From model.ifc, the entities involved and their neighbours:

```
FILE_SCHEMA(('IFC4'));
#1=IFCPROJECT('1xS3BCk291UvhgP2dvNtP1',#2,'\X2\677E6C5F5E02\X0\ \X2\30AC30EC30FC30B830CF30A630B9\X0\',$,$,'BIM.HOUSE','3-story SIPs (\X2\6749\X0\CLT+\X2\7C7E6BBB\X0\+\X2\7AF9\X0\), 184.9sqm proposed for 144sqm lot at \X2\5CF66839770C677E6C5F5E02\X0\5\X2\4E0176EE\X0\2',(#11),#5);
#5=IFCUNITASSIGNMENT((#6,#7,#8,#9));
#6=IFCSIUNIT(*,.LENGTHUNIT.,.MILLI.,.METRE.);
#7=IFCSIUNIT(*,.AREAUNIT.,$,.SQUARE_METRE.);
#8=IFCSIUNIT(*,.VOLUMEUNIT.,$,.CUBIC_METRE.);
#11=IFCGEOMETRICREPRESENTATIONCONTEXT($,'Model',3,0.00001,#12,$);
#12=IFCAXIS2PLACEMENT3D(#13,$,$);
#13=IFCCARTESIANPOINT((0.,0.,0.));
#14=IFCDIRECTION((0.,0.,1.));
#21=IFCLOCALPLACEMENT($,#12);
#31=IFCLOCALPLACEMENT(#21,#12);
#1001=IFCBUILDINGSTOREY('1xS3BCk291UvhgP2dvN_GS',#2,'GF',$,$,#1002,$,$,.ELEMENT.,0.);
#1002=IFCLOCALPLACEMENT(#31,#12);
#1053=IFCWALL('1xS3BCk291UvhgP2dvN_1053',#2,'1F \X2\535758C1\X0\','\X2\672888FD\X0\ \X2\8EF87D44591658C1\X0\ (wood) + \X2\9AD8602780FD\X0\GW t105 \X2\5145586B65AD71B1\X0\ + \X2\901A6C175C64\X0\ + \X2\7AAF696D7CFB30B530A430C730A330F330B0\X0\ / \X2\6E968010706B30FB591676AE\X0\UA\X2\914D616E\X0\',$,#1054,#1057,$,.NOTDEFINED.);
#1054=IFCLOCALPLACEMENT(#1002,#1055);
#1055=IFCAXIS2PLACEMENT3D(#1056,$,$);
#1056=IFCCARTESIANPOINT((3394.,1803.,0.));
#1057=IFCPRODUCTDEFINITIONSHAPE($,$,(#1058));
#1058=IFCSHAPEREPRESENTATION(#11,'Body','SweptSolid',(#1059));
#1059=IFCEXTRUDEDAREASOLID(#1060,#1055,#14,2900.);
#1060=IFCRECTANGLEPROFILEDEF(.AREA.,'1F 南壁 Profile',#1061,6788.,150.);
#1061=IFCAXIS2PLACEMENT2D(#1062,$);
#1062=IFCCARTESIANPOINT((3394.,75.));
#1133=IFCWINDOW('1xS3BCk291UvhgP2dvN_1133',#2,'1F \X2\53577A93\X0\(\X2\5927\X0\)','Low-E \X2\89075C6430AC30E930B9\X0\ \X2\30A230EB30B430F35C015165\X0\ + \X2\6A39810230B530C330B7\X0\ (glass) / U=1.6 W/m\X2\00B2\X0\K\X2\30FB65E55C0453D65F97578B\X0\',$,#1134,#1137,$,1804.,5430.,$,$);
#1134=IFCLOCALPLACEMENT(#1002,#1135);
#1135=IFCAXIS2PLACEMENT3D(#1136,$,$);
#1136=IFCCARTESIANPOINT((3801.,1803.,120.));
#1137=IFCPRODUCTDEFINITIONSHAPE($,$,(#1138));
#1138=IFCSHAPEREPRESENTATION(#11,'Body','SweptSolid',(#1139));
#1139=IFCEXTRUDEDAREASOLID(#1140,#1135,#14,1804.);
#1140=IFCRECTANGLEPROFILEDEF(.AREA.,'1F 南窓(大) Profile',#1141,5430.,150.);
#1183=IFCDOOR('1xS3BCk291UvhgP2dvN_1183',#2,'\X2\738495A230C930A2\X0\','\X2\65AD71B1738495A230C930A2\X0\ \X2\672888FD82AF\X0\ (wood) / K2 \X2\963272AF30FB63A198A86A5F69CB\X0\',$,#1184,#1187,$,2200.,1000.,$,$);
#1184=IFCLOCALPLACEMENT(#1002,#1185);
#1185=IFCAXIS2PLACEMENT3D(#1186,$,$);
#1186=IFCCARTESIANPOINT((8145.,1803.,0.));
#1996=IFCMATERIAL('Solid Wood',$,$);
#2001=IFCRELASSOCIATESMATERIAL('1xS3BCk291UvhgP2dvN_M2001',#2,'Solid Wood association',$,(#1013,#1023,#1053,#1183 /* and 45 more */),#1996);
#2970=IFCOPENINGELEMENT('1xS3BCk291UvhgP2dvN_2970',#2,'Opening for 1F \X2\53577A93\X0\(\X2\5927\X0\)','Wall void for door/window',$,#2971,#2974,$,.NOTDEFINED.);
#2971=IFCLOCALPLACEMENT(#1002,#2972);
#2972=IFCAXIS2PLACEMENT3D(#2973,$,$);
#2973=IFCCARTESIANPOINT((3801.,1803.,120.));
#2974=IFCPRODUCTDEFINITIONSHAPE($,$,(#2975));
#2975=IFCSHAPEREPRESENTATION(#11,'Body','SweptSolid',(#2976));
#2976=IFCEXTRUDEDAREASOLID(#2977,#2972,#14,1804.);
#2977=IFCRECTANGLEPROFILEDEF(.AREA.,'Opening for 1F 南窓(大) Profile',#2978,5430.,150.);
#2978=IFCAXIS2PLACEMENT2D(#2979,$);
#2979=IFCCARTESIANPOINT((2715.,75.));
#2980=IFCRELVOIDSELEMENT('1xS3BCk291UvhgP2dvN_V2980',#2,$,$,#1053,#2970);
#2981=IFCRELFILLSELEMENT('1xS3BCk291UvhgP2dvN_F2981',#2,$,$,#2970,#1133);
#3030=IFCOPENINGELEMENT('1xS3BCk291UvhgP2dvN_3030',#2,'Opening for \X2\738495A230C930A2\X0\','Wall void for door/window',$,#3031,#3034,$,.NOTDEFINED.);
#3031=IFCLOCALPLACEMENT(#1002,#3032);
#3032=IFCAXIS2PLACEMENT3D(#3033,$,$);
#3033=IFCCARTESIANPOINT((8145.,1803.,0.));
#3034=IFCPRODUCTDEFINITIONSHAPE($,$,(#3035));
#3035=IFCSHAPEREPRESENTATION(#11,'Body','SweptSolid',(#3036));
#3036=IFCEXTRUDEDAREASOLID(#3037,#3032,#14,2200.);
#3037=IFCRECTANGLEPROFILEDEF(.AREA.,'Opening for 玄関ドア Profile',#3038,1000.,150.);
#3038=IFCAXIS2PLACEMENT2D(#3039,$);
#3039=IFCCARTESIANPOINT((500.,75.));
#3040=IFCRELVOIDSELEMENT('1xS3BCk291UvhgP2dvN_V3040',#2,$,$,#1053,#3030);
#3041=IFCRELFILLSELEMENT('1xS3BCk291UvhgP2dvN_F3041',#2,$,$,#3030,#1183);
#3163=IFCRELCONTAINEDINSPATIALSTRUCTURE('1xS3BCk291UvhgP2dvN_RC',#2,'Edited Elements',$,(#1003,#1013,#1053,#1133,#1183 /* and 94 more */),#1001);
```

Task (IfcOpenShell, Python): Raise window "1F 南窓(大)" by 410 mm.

```python
import numpy as np
import ifcopenshell
import ifcopenshell.api.geometry
import ifcopenshell.util.placement
import ifcopenshell.util.unit

model = ifcopenshell.open("model.ifc")
unit_scale = ifcopenshell.util.unit.calculate_unit_scale(model)

window = model.by_guid("1xS3BCk291UvhgP2dvN_1133")
opening = window.FillsVoids[0].RelatingOpeningElement
dz = 0.41 / unit_scale

shift = np.array([0.0, 0.0, dz])
# The window is not placed relative to its opening, so move both.
for product in (opening, window):
    matrix = ifcopenshell.util.placement.get_local_placement(product.ObjectPlacement)
    matrix[:3, 3] += shift
    ifcopenshell.api.geometry.edit_object_placement(model, product=product, matrix=matrix, is_si=False)

print(f"moved by {dz * unit_scale:+.3f} m")

model.write("model-out.ifc")
```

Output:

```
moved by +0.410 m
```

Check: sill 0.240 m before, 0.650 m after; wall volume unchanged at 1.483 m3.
